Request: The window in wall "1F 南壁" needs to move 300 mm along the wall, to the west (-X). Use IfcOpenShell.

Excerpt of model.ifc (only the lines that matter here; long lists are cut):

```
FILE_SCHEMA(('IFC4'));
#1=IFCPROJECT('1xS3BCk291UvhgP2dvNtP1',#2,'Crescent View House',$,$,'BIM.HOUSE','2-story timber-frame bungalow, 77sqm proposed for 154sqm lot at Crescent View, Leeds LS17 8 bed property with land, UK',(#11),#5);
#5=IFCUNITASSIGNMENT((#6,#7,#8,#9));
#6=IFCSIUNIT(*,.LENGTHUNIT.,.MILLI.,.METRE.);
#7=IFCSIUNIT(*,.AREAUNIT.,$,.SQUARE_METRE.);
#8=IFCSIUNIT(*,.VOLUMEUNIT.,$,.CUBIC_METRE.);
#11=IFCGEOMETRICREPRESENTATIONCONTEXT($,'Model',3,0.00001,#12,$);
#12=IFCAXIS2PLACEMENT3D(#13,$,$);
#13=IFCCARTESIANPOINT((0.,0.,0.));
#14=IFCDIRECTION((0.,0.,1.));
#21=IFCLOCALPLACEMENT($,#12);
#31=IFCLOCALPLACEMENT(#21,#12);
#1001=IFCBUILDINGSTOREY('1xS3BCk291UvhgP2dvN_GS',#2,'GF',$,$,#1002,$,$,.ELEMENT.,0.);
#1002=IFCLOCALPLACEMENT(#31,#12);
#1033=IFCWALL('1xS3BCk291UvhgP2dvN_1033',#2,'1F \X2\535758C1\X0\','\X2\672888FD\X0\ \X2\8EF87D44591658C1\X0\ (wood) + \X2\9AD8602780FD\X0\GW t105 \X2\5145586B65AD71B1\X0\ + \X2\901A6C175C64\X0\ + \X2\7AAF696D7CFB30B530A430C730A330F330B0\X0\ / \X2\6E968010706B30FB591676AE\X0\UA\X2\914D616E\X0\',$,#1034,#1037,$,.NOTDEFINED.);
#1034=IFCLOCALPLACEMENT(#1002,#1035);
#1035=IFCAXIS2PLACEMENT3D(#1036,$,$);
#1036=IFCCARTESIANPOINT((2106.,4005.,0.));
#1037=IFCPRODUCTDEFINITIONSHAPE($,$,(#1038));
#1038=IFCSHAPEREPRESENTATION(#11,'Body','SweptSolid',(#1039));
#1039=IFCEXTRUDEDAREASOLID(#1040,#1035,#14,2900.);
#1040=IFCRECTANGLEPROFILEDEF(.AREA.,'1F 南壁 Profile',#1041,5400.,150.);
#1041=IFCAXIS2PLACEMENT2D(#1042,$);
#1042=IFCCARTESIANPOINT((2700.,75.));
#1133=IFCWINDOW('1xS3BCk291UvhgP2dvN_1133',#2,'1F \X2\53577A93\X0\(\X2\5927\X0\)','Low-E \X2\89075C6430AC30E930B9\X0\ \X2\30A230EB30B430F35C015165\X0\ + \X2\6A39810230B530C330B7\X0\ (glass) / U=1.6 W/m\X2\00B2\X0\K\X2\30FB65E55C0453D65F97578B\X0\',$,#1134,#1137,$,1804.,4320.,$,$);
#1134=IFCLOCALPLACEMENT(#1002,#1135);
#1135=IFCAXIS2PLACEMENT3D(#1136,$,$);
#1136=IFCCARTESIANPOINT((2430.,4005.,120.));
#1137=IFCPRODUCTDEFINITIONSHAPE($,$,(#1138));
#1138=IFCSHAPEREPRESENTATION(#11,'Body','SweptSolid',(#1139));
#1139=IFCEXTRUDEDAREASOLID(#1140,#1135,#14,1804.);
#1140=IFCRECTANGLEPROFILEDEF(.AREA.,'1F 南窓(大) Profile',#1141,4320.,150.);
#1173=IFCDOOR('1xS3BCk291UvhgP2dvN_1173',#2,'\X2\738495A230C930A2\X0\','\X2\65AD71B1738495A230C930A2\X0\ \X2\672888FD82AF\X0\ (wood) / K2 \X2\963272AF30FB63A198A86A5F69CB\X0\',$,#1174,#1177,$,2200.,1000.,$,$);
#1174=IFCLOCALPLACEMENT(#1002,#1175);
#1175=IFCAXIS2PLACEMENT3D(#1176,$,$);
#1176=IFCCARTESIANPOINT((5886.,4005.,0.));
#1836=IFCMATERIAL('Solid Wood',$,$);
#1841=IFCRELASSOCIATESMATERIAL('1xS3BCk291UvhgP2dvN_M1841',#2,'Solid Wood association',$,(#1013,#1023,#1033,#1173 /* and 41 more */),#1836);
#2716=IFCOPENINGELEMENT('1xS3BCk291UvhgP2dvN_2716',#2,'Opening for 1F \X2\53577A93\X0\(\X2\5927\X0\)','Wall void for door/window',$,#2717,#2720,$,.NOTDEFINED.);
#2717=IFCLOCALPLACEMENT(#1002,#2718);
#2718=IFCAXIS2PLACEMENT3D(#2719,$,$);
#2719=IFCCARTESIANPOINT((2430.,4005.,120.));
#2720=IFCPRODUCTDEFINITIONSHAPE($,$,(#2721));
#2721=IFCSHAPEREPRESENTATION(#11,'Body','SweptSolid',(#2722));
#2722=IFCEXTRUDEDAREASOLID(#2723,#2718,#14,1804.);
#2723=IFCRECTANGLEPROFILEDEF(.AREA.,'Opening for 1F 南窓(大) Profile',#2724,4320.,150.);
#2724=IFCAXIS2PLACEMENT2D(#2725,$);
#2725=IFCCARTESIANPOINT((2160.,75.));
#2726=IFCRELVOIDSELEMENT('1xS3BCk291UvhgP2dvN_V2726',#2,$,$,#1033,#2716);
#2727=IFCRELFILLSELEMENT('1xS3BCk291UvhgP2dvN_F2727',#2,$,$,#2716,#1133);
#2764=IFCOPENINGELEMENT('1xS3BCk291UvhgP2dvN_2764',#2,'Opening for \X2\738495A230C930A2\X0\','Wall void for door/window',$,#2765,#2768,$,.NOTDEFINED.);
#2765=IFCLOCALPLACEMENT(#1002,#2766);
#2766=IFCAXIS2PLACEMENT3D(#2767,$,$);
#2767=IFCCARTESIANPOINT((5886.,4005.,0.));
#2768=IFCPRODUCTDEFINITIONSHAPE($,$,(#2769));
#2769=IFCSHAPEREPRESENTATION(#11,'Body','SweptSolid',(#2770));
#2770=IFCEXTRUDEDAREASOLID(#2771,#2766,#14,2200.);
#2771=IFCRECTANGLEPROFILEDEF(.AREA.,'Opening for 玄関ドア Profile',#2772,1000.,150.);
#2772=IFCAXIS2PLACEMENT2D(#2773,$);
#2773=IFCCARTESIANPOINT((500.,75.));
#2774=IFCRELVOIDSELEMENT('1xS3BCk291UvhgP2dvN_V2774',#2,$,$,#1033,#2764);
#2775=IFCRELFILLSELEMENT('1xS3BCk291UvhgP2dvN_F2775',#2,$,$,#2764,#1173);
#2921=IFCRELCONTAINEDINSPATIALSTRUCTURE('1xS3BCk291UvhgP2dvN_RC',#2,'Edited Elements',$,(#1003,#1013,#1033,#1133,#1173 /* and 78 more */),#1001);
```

```python
import ifcopenshell
import ifcopenshell.api.geometry
import ifcopenshell.util.placement

model = ifcopenshell.open("model.ifc")

window = model.by_guid("1xS3BCk291UvhgP2dvN_1133")
opening = window.FillsVoids[0].RelatingOpeningElement
wall = opening.VoidsElements[0].RelatingBuildingElement

wall_matrix = ifcopenshell.util.placement.get_local_placement(wall.ObjectPlacement)
shift = wall_matrix[:3, 0] * -300.0
before = ifcopenshell.util.placement.get_local_placement(window.ObjectPlacement)[:3, 3].copy()

# The window is not placed relative to its opening, so move both.
for product in (opening, window):
    matrix = ifcopenshell.util.placement.get_local_placement(product.ObjectPlacement)
    matrix[:3, 3] += shift
    ifcopenshell.api.geometry.edit_object_placement(model, product=product, matrix=matrix, is_si=False)

after = ifcopenshell.util.placement.get_local_placement(window.ObjectPlacement)[:3, 3]
print("window moved by", (after - before).round(3) + 0.0)

model.write("model_rev.ifc")
```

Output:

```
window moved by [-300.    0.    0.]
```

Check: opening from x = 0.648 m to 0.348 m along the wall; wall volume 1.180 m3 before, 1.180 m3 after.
